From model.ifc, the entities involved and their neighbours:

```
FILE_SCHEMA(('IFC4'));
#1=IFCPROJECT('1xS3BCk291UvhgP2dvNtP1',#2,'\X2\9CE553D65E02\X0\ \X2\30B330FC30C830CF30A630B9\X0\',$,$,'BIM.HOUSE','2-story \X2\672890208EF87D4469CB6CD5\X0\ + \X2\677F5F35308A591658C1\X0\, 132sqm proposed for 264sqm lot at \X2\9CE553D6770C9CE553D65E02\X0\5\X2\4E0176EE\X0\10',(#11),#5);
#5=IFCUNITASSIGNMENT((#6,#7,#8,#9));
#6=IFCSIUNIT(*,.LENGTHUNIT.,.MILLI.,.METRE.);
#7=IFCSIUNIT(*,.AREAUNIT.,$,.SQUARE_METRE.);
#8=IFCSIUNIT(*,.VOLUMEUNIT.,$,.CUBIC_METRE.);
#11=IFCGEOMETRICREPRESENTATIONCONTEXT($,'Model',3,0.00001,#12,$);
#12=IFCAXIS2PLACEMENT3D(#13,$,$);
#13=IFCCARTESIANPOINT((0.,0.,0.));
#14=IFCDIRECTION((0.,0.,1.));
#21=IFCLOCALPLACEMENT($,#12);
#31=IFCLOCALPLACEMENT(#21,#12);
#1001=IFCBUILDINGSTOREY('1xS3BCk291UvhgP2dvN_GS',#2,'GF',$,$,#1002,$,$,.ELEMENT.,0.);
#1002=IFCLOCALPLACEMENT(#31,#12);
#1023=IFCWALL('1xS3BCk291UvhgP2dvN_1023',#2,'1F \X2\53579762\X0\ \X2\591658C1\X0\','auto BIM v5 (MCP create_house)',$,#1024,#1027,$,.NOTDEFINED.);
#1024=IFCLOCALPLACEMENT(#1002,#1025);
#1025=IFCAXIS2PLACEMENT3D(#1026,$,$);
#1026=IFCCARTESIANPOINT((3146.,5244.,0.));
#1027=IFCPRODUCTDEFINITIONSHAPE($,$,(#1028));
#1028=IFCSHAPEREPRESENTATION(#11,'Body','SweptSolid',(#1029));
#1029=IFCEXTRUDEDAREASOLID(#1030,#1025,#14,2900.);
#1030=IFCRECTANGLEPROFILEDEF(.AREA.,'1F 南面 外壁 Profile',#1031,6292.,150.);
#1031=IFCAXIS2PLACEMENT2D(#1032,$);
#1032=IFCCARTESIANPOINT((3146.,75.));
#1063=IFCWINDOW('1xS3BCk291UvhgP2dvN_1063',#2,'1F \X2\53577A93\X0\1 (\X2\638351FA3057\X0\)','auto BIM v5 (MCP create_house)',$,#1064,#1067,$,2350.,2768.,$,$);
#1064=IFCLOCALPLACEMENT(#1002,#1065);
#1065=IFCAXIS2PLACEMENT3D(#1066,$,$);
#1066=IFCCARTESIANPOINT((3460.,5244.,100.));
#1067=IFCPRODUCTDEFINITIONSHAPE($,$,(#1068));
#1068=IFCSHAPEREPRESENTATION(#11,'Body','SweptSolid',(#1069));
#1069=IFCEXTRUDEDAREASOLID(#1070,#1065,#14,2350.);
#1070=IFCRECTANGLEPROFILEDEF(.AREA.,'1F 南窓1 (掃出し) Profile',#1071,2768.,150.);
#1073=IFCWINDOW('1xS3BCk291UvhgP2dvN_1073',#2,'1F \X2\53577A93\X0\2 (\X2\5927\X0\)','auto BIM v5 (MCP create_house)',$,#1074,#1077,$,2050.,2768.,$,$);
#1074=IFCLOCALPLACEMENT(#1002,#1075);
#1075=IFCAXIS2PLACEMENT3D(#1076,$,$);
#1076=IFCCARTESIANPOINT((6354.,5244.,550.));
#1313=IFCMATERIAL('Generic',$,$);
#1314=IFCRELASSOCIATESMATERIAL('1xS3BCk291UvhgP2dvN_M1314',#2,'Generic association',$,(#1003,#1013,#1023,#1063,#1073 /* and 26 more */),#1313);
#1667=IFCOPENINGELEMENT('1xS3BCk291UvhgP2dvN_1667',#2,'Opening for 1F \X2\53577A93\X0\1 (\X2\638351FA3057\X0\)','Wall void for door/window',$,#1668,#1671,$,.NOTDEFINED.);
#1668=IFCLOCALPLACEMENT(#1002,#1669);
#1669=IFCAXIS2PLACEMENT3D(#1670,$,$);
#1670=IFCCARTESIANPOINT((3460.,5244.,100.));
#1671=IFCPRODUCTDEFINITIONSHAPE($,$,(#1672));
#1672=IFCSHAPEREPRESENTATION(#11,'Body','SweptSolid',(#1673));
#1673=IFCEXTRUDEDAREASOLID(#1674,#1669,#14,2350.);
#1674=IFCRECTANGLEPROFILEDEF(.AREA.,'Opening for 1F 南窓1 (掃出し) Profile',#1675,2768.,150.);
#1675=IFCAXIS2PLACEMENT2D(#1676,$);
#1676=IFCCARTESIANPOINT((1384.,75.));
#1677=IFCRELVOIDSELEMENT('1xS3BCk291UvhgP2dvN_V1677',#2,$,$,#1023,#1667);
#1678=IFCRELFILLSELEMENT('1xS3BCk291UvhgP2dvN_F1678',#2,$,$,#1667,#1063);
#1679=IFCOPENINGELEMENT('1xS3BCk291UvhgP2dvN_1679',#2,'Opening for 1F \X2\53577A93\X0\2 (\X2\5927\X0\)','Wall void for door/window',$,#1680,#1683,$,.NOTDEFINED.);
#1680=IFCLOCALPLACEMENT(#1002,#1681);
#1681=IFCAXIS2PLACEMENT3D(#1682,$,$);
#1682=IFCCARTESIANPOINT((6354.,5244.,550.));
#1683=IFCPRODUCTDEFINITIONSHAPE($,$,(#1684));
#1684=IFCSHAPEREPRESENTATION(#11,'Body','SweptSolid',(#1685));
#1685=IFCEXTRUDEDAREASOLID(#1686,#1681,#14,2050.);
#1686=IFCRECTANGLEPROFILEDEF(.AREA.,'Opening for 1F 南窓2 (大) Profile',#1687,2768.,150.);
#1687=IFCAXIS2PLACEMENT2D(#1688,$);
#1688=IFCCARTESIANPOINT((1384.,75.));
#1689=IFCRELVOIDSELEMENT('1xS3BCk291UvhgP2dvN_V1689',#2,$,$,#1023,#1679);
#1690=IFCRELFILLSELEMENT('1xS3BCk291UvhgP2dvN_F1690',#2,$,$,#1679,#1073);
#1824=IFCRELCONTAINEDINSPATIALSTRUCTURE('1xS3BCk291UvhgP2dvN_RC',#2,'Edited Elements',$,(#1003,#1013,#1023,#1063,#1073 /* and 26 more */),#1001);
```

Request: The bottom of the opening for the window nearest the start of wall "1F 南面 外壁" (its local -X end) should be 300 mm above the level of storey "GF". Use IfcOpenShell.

```python
import numpy as np
import ifcopenshell
import ifcopenshell.api.geometry
import ifcopenshell.geom
import ifcopenshell.util.element
import ifcopenshell.util.placement
import ifcopenshell.util.shape
import ifcopenshell.util.unit

model = ifcopenshell.open("model.ifc")
unit_scale = ifcopenshell.util.unit.calculate_unit_scale(model)

window = model.by_id(1063)
opening = window.FillsVoids[0].RelatingOpeningElement
storey = ifcopenshell.util.element.get_container(window, ifc_class="IfcBuildingStorey")
level = ifcopenshell.util.placement.get_local_placement(storey.ObjectPlacement)[2, 3]

# The opening's origin need not be at the sill, so measure its lowest point.
shape = ifcopenshell.geom.create_shape(ifcopenshell.geom.settings(), opening)
bottom = ifcopenshell.util.shape.get_shape_bottom_elevation(shape, shape.geometry) / unit_scale
dz = level + 0.3 / unit_scale - bottom

shift = np.array([0.0, 0.0, dz])
# The window is not placed relative to its opening, so move both.
for product in (opening, window):
    matrix = ifcopenshell.util.placement.get_local_placement(product.ObjectPlacement)
    matrix[:3, 3] += shift
    ifcopenshell.api.geometry.edit_object_placement(model, product=product, matrix=matrix, is_si=False)

print(f"moved by {dz * unit_scale:+.3f} m")

model.write("model_updated.ifc")
```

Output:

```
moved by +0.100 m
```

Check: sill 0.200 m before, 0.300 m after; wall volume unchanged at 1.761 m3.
